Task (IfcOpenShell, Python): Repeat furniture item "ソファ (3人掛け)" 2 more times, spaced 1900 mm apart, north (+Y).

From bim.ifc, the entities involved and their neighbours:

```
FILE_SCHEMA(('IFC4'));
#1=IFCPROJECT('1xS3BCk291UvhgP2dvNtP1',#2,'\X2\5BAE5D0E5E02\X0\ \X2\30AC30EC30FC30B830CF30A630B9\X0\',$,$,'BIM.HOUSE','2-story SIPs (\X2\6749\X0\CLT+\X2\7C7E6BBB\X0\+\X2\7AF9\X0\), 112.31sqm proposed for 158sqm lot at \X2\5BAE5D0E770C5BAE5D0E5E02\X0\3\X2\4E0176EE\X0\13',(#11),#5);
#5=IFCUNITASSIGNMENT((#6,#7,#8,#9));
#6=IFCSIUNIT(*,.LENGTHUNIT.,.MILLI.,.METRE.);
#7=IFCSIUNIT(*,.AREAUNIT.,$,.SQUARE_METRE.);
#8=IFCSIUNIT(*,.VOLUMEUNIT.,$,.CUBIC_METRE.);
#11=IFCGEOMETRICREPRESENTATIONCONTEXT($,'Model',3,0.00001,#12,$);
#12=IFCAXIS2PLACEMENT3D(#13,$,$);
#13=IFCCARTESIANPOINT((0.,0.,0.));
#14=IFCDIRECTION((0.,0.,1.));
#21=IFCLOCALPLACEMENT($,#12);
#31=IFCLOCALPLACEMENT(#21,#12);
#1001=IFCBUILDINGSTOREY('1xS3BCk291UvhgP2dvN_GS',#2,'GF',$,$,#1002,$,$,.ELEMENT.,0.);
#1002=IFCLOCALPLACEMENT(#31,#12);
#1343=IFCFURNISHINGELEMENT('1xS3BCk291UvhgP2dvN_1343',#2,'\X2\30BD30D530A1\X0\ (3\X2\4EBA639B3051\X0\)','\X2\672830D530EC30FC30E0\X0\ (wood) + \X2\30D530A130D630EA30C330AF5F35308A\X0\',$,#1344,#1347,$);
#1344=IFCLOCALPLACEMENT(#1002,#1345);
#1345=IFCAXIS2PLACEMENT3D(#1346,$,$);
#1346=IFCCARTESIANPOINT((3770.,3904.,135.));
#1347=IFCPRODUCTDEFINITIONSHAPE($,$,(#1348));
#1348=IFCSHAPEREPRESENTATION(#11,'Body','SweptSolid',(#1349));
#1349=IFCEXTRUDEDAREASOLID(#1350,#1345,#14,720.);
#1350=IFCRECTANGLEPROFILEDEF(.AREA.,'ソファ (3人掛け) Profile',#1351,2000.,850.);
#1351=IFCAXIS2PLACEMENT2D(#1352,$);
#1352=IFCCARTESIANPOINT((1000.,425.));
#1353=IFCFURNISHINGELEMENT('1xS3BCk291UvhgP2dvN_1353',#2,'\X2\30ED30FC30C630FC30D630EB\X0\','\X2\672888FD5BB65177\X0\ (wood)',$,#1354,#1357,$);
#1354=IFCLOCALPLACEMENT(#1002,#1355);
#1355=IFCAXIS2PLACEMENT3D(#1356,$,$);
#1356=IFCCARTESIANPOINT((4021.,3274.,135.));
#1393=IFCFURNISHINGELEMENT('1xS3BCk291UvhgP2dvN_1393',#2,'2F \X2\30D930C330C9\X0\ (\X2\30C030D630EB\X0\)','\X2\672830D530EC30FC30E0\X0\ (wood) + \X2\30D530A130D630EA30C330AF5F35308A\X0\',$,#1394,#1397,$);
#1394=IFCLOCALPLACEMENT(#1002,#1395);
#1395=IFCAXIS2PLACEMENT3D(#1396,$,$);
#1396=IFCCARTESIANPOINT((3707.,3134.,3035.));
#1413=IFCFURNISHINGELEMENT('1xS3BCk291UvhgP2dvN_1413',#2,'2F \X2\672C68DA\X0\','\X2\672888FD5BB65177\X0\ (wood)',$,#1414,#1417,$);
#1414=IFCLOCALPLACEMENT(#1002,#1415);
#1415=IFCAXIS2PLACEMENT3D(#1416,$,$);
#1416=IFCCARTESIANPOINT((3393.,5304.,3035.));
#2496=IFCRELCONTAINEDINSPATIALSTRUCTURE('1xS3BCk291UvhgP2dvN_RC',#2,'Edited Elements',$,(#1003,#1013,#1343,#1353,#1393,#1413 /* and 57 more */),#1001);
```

```python
import numpy as np
import ifcopenshell
import ifcopenshell.api.geometry
import ifcopenshell.api.root
import ifcopenshell.util.element
import ifcopenshell.util.placement
import ifcopenshell.util.unit

model = ifcopenshell.open("bim.ifc")
unit_scale = ifcopenshell.util.unit.calculate_unit_scale(model)


def reuse_history(source, copy):
    """copy_class also copies each property set's owner history, people and application; keep the originals."""
    for rel in copy.IsDefinedBy:
        if rel.is_a("IfcRelDefinesByProperties") and (history := rel.RelatingPropertyDefinition.OwnerHistory):
            rel.RelatingPropertyDefinition.OwnerHistory = source.OwnerHistory
            ifcopenshell.util.element.remove_deep2(model, history)


source = model.by_guid("1xS3BCk291UvhgP2dvN_1343")
base = ifcopenshell.util.placement.get_local_placement(source.ObjectPlacement)
step = np.array([0.0, 1.0, 0.0]) * 1.9 / unit_scale

for i in range(1, 3):
    copy = ifcopenshell.api.root.copy_class(model, product=source)
    copy.Representation = ifcopenshell.util.element.copy_deep(
        model, source.Representation, exclude=["IfcGeometricRepresentationContext", "IfcRepresentationMap"]
    )
    reuse_history(source, copy)
    matrix = base.copy()
    matrix[:3, 3] += i * step
    print("added at", matrix[:3, 3].round(3) + 0.0)
    ifcopenshell.api.geometry.edit_object_placement(model, product=copy, matrix=matrix, is_si=False)

model.write("bim_rev.ifc")
```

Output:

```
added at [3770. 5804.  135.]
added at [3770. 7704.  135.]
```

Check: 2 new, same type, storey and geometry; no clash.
